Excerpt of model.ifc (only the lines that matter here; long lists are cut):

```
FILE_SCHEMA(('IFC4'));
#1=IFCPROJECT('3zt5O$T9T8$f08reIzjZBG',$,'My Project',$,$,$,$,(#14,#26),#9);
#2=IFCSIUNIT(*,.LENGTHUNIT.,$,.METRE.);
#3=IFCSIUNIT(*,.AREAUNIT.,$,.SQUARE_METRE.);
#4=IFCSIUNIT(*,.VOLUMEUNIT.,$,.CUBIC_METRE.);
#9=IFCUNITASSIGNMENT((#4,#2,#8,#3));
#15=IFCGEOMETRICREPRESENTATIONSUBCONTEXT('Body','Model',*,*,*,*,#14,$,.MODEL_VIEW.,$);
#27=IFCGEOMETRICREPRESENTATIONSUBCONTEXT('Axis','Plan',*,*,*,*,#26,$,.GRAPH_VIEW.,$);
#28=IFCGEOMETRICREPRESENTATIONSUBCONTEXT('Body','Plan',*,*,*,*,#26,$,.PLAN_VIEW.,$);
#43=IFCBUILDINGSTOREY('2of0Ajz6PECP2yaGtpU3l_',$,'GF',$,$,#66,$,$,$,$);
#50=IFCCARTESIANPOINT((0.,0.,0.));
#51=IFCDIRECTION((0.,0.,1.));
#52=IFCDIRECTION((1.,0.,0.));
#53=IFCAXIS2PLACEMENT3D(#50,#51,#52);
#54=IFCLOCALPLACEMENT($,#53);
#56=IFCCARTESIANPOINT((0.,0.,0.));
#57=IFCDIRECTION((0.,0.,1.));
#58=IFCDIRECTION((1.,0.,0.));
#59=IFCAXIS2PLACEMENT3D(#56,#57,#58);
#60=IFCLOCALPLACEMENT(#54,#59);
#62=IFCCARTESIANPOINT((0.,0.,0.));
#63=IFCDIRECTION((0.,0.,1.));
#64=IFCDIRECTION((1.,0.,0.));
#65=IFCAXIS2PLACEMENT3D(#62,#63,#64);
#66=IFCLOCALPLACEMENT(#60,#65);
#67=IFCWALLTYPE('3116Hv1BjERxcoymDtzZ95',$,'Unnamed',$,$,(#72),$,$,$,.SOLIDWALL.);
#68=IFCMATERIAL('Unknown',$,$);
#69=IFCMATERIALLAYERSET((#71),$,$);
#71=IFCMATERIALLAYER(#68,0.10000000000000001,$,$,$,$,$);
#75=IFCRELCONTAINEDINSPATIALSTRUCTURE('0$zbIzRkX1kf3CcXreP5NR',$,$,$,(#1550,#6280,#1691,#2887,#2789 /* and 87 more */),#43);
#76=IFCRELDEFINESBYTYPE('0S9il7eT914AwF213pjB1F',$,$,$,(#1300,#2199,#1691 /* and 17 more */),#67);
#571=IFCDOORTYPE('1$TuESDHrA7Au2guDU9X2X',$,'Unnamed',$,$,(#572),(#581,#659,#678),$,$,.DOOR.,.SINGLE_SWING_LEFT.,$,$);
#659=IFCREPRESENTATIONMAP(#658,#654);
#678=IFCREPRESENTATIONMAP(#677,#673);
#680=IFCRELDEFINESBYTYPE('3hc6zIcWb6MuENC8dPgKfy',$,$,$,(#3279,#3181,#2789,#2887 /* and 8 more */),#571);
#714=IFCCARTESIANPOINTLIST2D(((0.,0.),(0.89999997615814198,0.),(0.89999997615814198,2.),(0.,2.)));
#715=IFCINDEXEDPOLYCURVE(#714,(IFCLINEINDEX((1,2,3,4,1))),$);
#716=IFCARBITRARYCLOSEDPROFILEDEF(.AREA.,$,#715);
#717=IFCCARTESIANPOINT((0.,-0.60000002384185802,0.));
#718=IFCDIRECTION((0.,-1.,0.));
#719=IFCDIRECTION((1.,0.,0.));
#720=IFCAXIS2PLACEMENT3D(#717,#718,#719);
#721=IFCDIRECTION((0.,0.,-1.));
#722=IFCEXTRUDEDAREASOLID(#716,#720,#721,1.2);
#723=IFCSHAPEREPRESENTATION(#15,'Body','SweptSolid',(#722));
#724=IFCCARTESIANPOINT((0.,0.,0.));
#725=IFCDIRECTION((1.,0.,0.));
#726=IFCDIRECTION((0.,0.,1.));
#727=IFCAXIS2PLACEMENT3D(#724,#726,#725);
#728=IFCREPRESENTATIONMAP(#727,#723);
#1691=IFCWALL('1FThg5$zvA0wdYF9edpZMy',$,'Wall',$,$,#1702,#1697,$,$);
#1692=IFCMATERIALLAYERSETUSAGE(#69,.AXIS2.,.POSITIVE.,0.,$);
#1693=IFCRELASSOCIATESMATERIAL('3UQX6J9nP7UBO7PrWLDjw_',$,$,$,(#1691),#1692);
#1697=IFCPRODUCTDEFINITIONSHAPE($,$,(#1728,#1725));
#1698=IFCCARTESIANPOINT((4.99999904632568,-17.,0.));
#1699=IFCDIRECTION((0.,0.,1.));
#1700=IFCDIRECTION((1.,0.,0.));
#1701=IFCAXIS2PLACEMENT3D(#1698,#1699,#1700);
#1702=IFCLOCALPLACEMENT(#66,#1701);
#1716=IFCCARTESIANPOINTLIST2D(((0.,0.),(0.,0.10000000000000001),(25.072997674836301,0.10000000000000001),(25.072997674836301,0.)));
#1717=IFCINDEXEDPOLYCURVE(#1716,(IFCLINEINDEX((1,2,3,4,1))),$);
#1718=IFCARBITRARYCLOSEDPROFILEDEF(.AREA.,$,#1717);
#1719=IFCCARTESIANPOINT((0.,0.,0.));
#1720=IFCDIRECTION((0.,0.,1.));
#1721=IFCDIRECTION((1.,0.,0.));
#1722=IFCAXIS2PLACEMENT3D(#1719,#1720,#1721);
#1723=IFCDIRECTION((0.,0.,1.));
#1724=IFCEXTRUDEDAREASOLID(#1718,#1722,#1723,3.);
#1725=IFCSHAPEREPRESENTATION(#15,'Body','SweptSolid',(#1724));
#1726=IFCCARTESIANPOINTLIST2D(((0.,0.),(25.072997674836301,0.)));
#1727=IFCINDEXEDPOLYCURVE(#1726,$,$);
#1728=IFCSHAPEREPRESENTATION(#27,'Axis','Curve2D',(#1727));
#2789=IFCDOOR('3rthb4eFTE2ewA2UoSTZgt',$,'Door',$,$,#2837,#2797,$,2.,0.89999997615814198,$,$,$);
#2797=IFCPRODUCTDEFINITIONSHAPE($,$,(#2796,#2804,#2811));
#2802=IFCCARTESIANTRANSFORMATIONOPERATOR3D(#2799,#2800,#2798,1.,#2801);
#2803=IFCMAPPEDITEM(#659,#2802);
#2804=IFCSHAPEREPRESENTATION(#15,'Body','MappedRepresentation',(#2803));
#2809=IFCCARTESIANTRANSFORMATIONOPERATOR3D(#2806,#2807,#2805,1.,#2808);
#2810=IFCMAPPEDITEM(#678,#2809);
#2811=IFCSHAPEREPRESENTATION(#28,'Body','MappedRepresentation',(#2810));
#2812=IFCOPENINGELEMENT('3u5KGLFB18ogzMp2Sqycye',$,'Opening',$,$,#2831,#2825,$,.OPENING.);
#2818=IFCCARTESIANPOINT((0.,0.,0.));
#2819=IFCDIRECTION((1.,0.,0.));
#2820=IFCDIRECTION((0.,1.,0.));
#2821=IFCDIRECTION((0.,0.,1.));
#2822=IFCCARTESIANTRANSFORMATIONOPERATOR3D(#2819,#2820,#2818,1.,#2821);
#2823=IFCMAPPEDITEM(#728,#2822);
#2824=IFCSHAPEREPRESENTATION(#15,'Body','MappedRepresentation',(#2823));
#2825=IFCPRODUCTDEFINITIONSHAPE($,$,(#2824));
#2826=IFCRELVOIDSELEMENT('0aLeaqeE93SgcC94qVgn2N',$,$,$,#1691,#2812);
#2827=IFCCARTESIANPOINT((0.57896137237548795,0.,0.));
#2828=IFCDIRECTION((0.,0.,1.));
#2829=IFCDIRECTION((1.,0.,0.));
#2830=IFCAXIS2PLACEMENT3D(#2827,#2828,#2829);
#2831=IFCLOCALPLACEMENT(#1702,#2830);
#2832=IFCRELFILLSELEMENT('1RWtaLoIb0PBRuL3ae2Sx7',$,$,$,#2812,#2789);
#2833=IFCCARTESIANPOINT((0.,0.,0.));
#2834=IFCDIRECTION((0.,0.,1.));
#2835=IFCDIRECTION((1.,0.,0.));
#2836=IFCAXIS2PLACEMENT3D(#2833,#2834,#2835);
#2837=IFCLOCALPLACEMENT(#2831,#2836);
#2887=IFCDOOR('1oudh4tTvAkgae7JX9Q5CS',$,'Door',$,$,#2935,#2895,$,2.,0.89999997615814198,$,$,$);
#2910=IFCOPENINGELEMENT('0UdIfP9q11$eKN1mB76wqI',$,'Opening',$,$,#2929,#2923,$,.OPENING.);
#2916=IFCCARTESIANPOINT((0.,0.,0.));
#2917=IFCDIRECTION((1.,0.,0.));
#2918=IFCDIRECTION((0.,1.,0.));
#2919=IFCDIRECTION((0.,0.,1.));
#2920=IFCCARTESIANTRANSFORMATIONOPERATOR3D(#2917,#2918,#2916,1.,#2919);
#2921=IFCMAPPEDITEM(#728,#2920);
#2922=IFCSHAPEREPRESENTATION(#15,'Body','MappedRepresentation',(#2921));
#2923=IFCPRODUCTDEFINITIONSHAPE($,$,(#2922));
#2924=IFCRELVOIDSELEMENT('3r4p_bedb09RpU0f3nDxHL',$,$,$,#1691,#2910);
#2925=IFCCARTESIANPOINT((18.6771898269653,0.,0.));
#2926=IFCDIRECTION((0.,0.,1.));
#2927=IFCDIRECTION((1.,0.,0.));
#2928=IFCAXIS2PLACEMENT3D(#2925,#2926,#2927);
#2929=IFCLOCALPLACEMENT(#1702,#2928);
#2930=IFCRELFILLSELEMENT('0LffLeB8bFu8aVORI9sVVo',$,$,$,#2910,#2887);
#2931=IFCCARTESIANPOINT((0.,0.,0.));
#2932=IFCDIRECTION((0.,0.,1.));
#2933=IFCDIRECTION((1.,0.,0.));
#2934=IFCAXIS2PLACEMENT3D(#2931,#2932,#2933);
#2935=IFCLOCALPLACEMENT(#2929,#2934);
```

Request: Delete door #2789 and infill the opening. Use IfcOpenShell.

```python
import ifcopenshell
import ifcopenshell.api.feature
import ifcopenshell.api.root
import ifcopenshell.geom
import ifcopenshell.util.shape

model = ifcopenshell.open("model.ifc")
settings = ifcopenshell.geom.settings()


def volume(element):
    """Net volume in cubic metres, openings subtracted."""
    shape = ifcopenshell.geom.create_shape(settings, element)
    return ifcopenshell.util.shape.get_volume(shape.geometry)


door = model.by_id(2789)
opening = door.FillsVoids[0].RelatingOpeningElement
wall = opening.VoidsElements[0].RelatingBuildingElement
before = volume(wall)

ifcopenshell.api.root.remove_product(model, product=door)
ifcopenshell.api.feature.remove_feature(model, feature=opening)

after = volume(wall)

print(f"wall volume {before:.3f} -> {after:.3f} m3")

model.write("model_edited.ifc")
```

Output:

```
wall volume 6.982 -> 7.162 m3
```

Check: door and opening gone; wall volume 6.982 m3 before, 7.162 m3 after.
